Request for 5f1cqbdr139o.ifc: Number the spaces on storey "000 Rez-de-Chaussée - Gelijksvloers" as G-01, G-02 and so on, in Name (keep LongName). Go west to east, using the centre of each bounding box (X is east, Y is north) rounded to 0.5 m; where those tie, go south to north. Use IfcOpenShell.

First a look at what the model holds.

```python
import ifcopenshell
import ifcopenshell.util.element
import ifcopenshell.util.placement

model = ifcopenshell.open("5f1cqbdr139o.ifc")
print(model.schema)
storey = next(s for s in model.by_type("IfcBuildingStorey") if s.Name == "000 Rez-de-Chaussée - Gelijksvloers")
spaces = [e for e in ifcopenshell.util.element.get_decomposition(storey) if e.is_a("IfcSpace")]
for e in sorted(spaces, key=lambda e: e.id()):
    origin = ifcopenshell.util.placement.get_local_placement(e.ObjectPlacement)[:3, 3]
    print(e.id(), e.Name, e.LongName, origin.round(2) + 0.0, sep=" | ")
```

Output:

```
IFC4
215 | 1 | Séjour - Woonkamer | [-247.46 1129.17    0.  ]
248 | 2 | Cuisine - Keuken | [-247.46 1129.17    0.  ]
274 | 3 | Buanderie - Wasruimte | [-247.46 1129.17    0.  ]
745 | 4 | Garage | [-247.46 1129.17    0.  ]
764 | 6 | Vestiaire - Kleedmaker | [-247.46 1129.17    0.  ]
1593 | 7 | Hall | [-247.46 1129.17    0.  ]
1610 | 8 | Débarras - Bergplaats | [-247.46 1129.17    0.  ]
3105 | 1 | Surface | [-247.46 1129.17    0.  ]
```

```python
import ifcopenshell
import ifcopenshell.geom
import ifcopenshell.util.element
import ifcopenshell.util.shape

model = ifcopenshell.open("5f1cqbdr139o.ifc")
settings = ifcopenshell.geom.settings()
settings.set("use-world-coords", True)


def centre(element):
    shape = ifcopenshell.geom.create_shape(settings, element)
    return ifcopenshell.util.shape.get_bbox_centroid(shape.geometry)


storey = next(s for s in model.by_type("IfcBuildingStorey") if s.Name == "000 Rez-de-Chaussée - Gelijksvloers")
spaces = [e for e in ifcopenshell.util.element.get_decomposition(storey) if e.is_a("IfcSpace")]

# Insertion points can sit at a corner or the storey origin, so sort by the geometry (in metres).
centres = {e: centre(e) for e in spaces}
spaces.sort(key=lambda e: (round(centres[e][0] / 0.5), centres[e][1]))

for i, e in enumerate(spaces, start=1):
    number = f"G-{i:02d}"
    e.Name = number
    print(e.id(), number)

model.write("5f1cqbdr139o_v2.ifc")
```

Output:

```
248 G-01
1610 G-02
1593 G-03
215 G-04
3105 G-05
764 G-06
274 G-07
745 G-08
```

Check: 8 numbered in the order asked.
